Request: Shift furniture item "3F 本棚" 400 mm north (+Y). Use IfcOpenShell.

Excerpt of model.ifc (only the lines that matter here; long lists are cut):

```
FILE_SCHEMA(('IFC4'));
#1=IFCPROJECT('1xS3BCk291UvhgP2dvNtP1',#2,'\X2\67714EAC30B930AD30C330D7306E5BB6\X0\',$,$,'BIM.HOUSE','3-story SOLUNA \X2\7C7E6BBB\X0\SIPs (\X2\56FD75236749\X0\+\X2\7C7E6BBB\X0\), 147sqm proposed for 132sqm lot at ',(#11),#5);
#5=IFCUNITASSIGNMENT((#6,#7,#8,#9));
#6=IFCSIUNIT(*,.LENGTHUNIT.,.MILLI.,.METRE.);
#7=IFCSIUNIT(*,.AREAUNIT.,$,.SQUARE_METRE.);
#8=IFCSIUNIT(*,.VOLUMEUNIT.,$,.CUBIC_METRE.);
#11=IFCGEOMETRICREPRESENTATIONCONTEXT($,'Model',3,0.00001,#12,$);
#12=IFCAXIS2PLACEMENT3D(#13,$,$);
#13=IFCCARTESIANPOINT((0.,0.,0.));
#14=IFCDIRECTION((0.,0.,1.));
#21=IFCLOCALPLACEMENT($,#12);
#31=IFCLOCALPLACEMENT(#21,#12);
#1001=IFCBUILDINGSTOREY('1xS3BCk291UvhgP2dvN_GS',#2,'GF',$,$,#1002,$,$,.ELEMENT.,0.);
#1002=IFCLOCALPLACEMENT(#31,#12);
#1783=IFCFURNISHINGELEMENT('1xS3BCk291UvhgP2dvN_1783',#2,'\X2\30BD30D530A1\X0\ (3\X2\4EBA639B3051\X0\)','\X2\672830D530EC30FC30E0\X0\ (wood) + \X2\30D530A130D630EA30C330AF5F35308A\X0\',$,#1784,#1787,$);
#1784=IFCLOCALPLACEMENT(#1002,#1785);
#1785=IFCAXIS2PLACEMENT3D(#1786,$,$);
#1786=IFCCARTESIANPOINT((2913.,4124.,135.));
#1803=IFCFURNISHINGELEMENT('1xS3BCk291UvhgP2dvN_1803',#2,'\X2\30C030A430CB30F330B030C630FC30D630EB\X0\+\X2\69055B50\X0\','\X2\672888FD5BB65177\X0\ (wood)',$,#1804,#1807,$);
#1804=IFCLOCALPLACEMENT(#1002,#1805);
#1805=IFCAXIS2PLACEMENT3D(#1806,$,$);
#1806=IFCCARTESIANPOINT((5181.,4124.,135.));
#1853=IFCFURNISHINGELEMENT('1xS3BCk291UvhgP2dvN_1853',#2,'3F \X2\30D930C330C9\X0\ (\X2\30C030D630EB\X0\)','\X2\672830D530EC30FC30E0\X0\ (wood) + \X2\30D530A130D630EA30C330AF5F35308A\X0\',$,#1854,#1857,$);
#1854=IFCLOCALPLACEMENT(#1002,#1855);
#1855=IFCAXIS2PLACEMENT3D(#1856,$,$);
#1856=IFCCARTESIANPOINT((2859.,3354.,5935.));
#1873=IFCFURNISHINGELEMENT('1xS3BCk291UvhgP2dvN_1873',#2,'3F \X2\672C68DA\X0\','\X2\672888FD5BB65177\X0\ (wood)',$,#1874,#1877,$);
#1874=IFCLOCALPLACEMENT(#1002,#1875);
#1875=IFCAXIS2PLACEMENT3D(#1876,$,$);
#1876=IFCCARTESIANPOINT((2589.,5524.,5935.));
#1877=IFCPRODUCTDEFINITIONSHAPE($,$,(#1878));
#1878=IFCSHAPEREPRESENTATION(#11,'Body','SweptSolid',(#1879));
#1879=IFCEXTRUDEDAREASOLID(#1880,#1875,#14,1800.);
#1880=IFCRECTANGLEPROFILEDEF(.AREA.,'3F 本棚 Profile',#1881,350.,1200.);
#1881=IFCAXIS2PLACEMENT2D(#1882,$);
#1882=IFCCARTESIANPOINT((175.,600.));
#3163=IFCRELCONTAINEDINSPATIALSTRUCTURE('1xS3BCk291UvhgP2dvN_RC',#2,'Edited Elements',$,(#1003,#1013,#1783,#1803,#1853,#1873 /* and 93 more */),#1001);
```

```python
import ifcopenshell
import ifcopenshell.api.geometry
import ifcopenshell.util.placement
import ifcopenshell.util.unit

model = ifcopenshell.open("model.ifc")
unit_scale = ifcopenshell.util.unit.calculate_unit_scale(model)

item = model.by_guid("1xS3BCk291UvhgP2dvN_1873")
matrix = ifcopenshell.util.placement.get_local_placement(item.ObjectPlacement)
matrix[1, 3] += 0.4 / unit_scale
ifcopenshell.api.geometry.edit_object_placement(model, product=item, matrix=matrix, is_si=False)

print(ifcopenshell.util.placement.get_local_placement(item.ObjectPlacement).round(3) + 0.0)

model.write("model_rev.ifc")
```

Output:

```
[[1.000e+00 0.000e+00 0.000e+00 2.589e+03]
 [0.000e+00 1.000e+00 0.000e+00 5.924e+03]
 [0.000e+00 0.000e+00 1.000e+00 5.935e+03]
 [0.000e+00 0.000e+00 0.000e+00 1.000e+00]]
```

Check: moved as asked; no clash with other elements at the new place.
